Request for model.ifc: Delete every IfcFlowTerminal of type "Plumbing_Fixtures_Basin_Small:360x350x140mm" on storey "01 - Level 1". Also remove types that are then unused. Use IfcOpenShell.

First a look at what the model holds.

```python
import ifcopenshell
import ifcopenshell.util.element

model = ifcopenshell.open("model.ifc")
print(model.schema)
storey = next(s for s in model.by_type("IfcBuildingStorey") if s.Name == "01 - Level 1")
terminals = [e for e in ifcopenshell.util.element.get_decomposition(storey) if e.is_a("IfcFlowTerminal")]
seen = {}
for e in terminals:
    element_type = ifcopenshell.util.element.get_type(e)
    name = element_type.Name if element_type not in (None, e) else None
    seen[name] = seen.get(name, 0) + 1
for name, count in sorted(seen.items(), key=str):
    print(count, "x", name)
```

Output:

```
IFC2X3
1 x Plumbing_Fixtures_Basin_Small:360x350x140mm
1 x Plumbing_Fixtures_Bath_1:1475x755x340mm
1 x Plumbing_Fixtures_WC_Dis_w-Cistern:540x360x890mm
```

```python
import ifcopenshell
import ifcopenshell.api.root
import ifcopenshell.util.element

model = ifcopenshell.open("model.ifc")

storey = next(s for s in model.by_type("IfcBuildingStorey") if s.Name == "01 - Level 1")
terminals = [e for e in ifcopenshell.util.element.get_decomposition(storey) if e.is_a("IfcFlowTerminal")]
targets = [e for e in terminals if (t := ifcopenshell.util.element.get_type(e)) not in (None, e) and t.Name == "Plumbing_Fixtures_Basin_Small:360x350x140mm"]
types = {ifcopenshell.util.element.get_type(e) for e in targets} - {None, *targets}

for e in targets:
    ifcopenshell.api.root.remove_product(model, product=e)
print(len(targets), "removed")

unused = [t for t in types if not ifcopenshell.util.element.get_types(t)]
for t in unused:
    ifcopenshell.api.root.remove_product(model, product=t)
print(len(unused), "unused types removed")

model.write("model_edited.ifc")
```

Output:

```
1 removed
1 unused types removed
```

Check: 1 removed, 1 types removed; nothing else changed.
